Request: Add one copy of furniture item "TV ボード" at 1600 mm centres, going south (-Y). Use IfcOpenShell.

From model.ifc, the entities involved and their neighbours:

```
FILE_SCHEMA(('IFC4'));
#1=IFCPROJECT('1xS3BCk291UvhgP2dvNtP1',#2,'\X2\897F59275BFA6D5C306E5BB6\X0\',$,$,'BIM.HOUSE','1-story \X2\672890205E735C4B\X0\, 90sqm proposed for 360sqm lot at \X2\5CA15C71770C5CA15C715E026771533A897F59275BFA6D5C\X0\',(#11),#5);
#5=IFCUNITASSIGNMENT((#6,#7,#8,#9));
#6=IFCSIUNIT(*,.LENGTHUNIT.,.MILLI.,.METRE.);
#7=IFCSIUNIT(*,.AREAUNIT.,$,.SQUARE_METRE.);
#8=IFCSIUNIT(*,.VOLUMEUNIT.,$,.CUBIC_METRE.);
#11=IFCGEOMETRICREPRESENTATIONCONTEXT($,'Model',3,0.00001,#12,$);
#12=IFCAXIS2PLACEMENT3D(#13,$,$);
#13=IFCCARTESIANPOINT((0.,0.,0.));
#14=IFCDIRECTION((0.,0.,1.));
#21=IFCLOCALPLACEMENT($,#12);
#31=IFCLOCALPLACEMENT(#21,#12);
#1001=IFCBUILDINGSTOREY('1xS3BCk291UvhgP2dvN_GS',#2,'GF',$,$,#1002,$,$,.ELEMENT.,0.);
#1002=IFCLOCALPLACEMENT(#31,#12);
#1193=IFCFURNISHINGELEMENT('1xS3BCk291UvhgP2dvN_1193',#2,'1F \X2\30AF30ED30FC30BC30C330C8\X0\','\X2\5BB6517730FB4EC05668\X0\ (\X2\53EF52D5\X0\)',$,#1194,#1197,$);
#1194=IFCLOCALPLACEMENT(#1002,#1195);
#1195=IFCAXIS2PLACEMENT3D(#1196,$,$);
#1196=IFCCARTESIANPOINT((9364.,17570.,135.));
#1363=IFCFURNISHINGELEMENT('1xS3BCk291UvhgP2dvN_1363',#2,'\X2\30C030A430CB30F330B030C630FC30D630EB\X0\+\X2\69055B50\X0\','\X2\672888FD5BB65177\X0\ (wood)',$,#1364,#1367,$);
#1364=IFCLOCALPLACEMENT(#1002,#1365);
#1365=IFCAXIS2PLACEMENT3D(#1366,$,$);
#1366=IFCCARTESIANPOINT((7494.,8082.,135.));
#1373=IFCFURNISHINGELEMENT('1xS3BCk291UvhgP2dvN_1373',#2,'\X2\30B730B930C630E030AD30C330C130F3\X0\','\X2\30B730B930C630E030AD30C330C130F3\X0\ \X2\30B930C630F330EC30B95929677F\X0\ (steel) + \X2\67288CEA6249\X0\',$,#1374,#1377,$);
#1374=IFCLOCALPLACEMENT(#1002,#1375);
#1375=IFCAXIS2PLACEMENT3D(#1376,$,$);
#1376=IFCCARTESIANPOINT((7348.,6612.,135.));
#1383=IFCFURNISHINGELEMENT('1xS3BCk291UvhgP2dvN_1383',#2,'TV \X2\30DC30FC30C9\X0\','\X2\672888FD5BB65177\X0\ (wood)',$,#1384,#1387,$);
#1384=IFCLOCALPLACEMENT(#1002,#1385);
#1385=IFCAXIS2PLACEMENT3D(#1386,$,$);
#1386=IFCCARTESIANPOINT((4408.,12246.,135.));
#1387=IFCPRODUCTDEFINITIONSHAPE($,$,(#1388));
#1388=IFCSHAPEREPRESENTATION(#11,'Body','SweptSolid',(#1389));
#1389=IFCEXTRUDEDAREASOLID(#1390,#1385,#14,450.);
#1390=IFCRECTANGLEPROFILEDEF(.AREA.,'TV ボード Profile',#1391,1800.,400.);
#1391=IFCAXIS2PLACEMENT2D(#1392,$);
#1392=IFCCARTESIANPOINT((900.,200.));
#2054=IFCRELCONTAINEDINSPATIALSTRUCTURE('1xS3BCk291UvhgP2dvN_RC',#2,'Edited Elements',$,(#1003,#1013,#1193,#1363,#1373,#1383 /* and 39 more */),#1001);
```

```python
import numpy as np
import ifcopenshell
import ifcopenshell.api.geometry
import ifcopenshell.api.root
import ifcopenshell.util.element
import ifcopenshell.util.placement

model = ifcopenshell.open("model.ifc")


def reuse_history(source, copy):
    """copy_class also copies each property set's owner history, people and application; keep the originals."""
    for rel in copy.IsDefinedBy:
        if rel.is_a("IfcRelDefinesByProperties") and (history := rel.RelatingPropertyDefinition.OwnerHistory):
            rel.RelatingPropertyDefinition.OwnerHistory = source.OwnerHistory
            ifcopenshell.util.element.remove_deep2(model, history)


source = model.by_guid("1xS3BCk291UvhgP2dvN_1383")
base = ifcopenshell.util.placement.get_local_placement(source.ObjectPlacement)
step = np.array([0.0, -1.0, 0.0]) * 1600.0

for i in range(1, 2):
    copy = ifcopenshell.api.root.copy_class(model, product=source)
    copy.Representation = ifcopenshell.util.element.copy_deep(
        model, source.Representation, exclude=["IfcGeometricRepresentationContext", "IfcRepresentationMap"]
    )
    reuse_history(source, copy)
    matrix = base.copy()
    matrix[:3, 3] += i * step
    print("added at", matrix[:3, 3].round(3) + 0.0)
    ifcopenshell.api.geometry.edit_object_placement(model, product=copy, matrix=matrix, is_si=False)

model.write("model_edited.ifc")
```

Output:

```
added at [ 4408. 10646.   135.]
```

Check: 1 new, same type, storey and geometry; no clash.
